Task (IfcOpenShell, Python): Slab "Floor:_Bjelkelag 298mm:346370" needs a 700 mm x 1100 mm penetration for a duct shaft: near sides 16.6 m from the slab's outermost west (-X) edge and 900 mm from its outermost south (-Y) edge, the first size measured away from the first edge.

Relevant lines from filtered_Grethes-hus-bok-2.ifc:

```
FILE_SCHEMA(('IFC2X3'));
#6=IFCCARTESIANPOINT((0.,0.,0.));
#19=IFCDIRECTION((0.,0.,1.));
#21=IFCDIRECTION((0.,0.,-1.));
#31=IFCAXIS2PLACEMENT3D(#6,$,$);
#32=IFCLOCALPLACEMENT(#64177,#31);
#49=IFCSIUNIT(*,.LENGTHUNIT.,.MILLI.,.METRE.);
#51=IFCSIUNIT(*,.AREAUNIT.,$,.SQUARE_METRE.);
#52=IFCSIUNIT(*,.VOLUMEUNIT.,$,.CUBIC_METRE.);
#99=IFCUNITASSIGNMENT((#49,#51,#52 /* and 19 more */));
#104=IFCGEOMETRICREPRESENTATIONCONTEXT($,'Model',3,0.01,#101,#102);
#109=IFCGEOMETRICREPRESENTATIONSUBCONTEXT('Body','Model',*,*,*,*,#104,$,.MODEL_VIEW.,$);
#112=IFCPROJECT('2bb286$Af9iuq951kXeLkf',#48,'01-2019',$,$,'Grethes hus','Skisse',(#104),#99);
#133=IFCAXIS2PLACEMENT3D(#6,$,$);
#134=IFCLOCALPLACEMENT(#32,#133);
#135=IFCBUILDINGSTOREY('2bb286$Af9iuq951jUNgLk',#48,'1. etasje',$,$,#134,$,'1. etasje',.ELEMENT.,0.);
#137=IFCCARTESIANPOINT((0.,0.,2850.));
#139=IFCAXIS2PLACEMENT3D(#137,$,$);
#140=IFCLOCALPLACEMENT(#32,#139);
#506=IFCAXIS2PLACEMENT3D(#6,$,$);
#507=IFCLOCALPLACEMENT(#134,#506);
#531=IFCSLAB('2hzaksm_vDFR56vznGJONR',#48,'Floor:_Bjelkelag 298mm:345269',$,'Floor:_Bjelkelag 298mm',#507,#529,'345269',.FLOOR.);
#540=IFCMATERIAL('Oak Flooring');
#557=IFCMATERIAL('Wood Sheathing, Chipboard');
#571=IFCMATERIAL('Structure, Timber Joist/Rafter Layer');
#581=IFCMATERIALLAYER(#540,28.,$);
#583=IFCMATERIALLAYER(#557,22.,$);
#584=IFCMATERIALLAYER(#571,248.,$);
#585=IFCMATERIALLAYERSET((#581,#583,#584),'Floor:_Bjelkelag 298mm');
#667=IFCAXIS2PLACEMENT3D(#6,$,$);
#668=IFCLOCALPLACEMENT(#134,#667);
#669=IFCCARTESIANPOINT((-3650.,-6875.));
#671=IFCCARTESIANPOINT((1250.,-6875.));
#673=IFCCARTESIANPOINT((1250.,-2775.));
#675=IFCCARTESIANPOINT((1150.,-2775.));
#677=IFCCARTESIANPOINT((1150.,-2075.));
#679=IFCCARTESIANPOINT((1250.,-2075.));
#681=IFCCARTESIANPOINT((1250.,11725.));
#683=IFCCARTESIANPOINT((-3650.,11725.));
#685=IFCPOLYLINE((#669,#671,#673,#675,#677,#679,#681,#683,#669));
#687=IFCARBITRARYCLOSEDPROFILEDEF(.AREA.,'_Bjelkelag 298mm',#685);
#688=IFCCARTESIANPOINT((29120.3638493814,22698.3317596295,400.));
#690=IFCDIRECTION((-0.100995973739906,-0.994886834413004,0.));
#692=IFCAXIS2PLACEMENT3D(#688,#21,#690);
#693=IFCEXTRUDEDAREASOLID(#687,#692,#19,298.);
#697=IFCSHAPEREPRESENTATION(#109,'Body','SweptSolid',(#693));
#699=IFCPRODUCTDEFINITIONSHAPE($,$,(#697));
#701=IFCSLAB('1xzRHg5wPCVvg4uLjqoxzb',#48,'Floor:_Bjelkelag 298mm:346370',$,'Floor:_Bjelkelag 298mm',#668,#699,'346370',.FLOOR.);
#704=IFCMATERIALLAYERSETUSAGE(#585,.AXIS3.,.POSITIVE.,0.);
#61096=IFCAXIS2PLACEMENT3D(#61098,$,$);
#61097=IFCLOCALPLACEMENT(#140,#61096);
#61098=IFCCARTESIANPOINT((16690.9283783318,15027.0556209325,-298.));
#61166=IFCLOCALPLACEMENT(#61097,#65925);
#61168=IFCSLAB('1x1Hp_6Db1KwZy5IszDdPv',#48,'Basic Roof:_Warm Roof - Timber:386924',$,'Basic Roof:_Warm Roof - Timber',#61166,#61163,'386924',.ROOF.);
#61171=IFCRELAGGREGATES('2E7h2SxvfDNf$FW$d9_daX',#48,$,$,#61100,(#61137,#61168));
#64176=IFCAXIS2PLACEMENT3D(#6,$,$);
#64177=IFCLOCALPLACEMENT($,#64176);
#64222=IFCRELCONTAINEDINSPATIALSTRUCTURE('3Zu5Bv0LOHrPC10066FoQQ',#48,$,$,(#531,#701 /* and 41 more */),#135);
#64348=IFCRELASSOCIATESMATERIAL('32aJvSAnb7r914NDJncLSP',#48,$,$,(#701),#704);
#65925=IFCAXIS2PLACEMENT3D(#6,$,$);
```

```python
import numpy as np
import ifcopenshell
import ifcopenshell.api.feature
import ifcopenshell.api.geometry
import ifcopenshell.api.root
import ifcopenshell.geom
import ifcopenshell.util.placement
import ifcopenshell.util.representation
import ifcopenshell.util.shape
import ifcopenshell.util.unit

model = ifcopenshell.open("filtered_Grethes-hus-bok-2.ifc")
unit_scale = ifcopenshell.util.unit.calculate_unit_scale(model)
settings = ifcopenshell.geom.settings()


def volume(element):
    """Net volume in cubic metres, openings subtracted."""
    shape = ifcopenshell.geom.create_shape(settings, element)
    return ifcopenshell.util.shape.get_volume(shape.geometry)


slab = model.by_guid("1xzRHg5wPCVvg4uLjqoxzb")
before = volume(slab)

# Extent in the slab's own axes, in metres. The edges named are its -X and -Y sides.
slab_shape = ifcopenshell.geom.create_shape(settings, slab)
vertices = ifcopenshell.util.shape.get_vertices(slab_shape.geometry)
x_min, y_min, bottom = vertices.min(axis=0)
top = vertices[:, 2].max()

opening = ifcopenshell.api.root.create_entity(model, ifc_class="IfcOpeningElement", name="Duct shaft opening")
context = ifcopenshell.util.representation.get_context(model, "Model", "Body", "MODEL_VIEW")
width, depth = 0.7, 1.1
outline = [(0.0, 0.0), (width, 0.0), (width, depth), (0.0, depth), (0.0, 0.0)]
# Overshoot both faces by 50 mm so the cut is clean.
shape = ifcopenshell.api.geometry.add_slab_representation(
    model, context=context, depth=top - bottom + 0.1, polyline=outline
)
ifcopenshell.api.geometry.assign_representation(model, product=opening, representation=shape)

matrix = ifcopenshell.util.placement.get_local_placement(slab.ObjectPlacement)
matrix[:, 3] = matrix @ np.append(np.array([x_min + 16.6, y_min + 0.9, bottom - 0.05]) / unit_scale, 1.0)
ifcopenshell.api.geometry.edit_object_placement(model, product=opening, matrix=matrix, is_si=False)
ifcopenshell.api.feature.add_feature(model, feature=opening, element=slab)

after = volume(slab)

print(f"slab volume {before:.3f} -> {after:.3f} m3")

model.write("filtered_Grethes-hus-bok-2_rev.ifc")
```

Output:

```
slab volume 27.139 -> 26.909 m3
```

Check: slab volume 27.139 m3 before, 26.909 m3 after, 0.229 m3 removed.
